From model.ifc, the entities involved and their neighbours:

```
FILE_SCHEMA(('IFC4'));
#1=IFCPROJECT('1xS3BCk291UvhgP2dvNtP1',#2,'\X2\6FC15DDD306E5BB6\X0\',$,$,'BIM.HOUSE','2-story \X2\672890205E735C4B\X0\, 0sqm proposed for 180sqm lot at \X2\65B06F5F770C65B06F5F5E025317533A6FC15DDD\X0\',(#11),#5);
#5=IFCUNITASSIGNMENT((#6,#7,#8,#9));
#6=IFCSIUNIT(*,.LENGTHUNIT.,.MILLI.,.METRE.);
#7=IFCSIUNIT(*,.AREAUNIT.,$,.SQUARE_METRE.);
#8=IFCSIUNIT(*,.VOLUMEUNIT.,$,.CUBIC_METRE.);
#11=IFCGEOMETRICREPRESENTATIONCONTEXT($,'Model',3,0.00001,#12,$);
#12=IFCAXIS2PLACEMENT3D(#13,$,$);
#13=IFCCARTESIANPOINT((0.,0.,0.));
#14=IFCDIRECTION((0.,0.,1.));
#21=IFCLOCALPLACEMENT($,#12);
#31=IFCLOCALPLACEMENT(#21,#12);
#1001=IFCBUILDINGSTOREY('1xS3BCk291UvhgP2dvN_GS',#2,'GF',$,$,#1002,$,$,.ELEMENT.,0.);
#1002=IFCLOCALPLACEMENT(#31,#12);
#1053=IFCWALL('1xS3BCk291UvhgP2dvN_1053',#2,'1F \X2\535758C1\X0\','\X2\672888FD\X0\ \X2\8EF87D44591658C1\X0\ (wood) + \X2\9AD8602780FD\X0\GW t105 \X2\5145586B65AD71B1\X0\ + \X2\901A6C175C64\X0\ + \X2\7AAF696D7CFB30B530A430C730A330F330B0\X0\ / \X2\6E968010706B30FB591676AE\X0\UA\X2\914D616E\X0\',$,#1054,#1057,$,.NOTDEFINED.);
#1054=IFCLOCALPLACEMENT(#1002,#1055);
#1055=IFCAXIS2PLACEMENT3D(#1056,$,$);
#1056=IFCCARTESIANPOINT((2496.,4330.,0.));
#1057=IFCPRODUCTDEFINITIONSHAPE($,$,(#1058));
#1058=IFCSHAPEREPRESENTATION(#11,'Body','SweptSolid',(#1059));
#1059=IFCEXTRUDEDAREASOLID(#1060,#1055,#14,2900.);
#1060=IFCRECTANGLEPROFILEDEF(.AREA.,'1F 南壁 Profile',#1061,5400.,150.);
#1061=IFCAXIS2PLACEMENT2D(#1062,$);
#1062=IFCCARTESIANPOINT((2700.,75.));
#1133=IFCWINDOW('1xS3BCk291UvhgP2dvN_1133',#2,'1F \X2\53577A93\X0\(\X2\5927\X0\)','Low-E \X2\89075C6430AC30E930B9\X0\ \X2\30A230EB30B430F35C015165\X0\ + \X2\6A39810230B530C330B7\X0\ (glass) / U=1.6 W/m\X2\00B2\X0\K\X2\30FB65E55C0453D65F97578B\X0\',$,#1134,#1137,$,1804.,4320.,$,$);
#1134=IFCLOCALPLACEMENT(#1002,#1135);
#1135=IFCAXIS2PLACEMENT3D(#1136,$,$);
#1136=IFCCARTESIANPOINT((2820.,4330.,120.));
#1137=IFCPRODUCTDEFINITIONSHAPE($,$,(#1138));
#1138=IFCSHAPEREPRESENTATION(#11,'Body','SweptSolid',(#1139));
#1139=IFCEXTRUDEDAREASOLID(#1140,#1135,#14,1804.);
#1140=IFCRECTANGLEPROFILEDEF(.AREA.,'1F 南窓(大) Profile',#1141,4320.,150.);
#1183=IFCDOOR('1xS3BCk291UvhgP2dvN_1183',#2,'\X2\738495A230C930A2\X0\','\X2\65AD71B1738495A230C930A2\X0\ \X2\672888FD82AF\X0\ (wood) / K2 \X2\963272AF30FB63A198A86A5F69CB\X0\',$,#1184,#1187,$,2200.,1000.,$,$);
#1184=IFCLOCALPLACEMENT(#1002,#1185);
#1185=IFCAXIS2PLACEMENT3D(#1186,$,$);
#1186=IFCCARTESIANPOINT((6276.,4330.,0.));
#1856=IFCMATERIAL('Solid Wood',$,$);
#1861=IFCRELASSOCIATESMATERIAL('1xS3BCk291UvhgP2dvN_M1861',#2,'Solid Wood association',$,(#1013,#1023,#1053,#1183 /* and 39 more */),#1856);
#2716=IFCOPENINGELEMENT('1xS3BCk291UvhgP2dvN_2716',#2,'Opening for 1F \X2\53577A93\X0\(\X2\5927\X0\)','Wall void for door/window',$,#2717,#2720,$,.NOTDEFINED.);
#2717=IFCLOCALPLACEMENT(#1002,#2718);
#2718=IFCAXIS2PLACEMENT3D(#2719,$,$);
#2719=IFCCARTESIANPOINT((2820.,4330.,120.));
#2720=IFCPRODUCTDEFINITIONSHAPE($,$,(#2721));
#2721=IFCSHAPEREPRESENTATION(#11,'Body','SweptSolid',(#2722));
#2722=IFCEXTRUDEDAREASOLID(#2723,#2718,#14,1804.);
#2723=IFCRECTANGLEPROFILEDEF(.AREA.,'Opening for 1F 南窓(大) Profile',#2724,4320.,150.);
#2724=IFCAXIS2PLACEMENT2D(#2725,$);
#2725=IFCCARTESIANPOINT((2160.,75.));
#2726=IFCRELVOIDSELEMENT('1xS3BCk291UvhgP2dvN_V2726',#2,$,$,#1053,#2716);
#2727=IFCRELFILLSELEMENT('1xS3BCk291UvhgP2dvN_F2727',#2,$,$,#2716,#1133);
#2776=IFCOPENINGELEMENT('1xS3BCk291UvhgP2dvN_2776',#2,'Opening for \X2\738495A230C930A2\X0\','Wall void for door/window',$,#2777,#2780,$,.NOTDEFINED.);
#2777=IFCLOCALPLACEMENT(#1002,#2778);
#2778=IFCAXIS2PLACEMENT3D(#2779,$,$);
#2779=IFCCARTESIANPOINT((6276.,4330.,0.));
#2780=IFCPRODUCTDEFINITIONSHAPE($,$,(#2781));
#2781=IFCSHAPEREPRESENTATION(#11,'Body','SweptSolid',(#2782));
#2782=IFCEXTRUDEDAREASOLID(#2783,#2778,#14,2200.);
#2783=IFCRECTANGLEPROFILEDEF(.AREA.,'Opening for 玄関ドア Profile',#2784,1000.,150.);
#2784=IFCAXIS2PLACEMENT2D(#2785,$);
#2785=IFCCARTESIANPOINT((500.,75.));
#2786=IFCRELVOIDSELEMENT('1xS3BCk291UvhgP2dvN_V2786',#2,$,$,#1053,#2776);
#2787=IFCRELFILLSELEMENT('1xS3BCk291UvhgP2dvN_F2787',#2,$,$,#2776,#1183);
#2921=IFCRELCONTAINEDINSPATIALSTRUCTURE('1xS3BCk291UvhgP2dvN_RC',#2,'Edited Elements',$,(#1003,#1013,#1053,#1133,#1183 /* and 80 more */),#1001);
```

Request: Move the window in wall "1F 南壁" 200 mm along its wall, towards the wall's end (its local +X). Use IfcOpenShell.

```python
import ifcopenshell
import ifcopenshell.api.geometry
import ifcopenshell.util.placement
import ifcopenshell.util.unit

model = ifcopenshell.open("model.ifc")
unit_scale = ifcopenshell.util.unit.calculate_unit_scale(model)

window = model.by_guid("1xS3BCk291UvhgP2dvN_1133")
opening = window.FillsVoids[0].RelatingOpeningElement
wall = opening.VoidsElements[0].RelatingBuildingElement

wall_matrix = ifcopenshell.util.placement.get_local_placement(wall.ObjectPlacement)
shift = wall_matrix[:3, 0] * 0.2 / unit_scale
before = ifcopenshell.util.placement.get_local_placement(window.ObjectPlacement)[:3, 3].copy()

# The window is not placed relative to its opening, so move both.
for product in (opening, window):
    matrix = ifcopenshell.util.placement.get_local_placement(product.ObjectPlacement)
    matrix[:3, 3] += shift
    ifcopenshell.api.geometry.edit_object_placement(model, product=product, matrix=matrix, is_si=False)

after = ifcopenshell.util.placement.get_local_placement(window.ObjectPlacement)[:3, 3]
print("window moved by", (after - before).round(3) + 0.0)

model.write("model_rev.ifc")
```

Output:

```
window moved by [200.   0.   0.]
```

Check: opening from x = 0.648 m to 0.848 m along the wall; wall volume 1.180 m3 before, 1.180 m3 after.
